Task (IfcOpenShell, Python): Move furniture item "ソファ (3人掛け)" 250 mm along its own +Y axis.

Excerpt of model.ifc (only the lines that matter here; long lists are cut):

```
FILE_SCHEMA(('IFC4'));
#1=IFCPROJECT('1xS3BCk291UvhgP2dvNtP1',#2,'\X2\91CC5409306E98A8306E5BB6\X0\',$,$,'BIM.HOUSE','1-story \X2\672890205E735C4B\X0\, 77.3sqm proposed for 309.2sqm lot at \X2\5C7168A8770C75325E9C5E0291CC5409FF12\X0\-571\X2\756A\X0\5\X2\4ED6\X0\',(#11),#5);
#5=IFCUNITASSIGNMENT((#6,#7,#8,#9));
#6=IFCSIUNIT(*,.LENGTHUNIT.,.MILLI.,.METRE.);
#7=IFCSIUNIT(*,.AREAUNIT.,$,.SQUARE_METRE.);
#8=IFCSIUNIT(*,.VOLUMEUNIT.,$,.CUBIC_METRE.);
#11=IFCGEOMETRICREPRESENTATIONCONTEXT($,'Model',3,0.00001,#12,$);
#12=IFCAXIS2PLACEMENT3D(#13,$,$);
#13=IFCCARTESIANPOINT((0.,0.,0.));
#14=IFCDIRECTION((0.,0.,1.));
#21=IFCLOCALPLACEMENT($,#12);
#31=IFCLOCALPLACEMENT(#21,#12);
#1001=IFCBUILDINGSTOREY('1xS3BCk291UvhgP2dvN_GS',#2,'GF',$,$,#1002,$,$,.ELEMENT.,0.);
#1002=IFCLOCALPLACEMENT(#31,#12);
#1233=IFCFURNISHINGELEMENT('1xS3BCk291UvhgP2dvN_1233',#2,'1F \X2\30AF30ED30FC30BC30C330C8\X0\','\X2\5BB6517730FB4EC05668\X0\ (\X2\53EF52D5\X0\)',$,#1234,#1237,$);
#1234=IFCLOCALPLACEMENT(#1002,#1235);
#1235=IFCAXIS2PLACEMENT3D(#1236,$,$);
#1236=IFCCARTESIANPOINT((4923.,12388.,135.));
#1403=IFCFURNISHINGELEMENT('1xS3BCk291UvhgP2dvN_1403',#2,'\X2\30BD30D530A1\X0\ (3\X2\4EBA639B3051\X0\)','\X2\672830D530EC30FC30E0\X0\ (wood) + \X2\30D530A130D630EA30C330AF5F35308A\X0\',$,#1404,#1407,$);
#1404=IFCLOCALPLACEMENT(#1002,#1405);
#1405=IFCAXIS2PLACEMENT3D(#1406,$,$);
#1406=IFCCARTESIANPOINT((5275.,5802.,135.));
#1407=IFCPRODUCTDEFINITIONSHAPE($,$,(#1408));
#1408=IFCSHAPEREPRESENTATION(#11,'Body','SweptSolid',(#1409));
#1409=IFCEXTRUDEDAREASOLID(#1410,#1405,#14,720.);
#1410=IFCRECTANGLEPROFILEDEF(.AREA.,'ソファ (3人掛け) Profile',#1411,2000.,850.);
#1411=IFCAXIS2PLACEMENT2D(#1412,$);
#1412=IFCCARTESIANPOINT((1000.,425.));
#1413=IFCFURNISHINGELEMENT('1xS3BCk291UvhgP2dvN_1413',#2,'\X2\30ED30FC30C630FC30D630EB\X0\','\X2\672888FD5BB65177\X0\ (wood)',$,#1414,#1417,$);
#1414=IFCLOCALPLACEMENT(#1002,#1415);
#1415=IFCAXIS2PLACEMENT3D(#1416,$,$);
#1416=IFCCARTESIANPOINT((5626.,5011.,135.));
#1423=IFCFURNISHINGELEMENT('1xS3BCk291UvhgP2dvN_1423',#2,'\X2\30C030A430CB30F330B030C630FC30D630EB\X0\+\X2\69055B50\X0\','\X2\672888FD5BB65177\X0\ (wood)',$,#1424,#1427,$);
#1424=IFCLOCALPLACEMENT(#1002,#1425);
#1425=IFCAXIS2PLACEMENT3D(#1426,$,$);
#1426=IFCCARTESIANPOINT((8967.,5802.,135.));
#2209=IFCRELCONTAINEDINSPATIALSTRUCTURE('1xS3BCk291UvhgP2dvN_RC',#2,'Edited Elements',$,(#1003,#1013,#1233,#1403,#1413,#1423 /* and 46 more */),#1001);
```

```python
import ifcopenshell
import ifcopenshell.api.geometry
import ifcopenshell.util.placement

model = ifcopenshell.open("model.ifc")

item = model.by_guid("1xS3BCk291UvhgP2dvN_1403")
matrix = ifcopenshell.util.placement.get_local_placement(item.ObjectPlacement)
matrix[:3, 3] += matrix[:3, 1] * 250.0
ifcopenshell.api.geometry.edit_object_placement(model, product=item, matrix=matrix, is_si=False)

print(ifcopenshell.util.placement.get_local_placement(item.ObjectPlacement).round(3) + 0.0)

model.write("model_edited.ifc")
```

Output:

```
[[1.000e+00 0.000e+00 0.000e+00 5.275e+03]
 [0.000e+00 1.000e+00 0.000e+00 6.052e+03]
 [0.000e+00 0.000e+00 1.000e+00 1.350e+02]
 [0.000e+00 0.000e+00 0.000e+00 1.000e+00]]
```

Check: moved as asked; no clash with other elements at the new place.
